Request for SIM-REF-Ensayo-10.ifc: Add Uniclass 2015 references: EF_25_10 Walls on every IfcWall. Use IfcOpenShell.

First a look at what the model holds.

```python
import ifcopenshell

model = ifcopenshell.open("SIM-REF-Ensayo-10.ifc")
print(model.schema)
print("classifications:", [c.Name for c in model.by_type("IfcClassification")])
for ifc_class in ("IfcDoor", "IfcRoof", "IfcStair", "IfcWall", "IfcWindow"):
    print(ifc_class, len(model.by_type(ifc_class)))
```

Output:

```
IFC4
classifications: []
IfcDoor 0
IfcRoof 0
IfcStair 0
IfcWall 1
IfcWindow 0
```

```python
import ifcopenshell
import ifcopenshell.api.classification

model = ifcopenshell.open("SIM-REF-Ensayo-10.ifc")

system = ifcopenshell.api.classification.add_classification(model, classification="Uniclass 2015")

codes = {
    "IfcWall": ("EF_25_10", "Walls"),
}
for ifc_class, (code, name) in codes.items():
    products = model.by_type(ifc_class)
    ifcopenshell.api.classification.add_reference(
        model, products=products, classification=system, identification=code, name=name
    )
    print(code, len(products))

model.write("SIM-REF-Ensayo-10-out.ifc")
```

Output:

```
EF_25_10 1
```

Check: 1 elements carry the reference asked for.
